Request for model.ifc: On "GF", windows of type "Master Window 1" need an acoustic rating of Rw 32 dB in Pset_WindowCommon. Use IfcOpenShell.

First a look at what the model holds.

```python
import ifcopenshell
import ifcopenshell.util.element

model = ifcopenshell.open("model.ifc")
print(model.schema)
storey = next(s for s in model.by_type("IfcBuildingStorey") if s.Name == "GF")
windows = [e for e in ifcopenshell.util.element.get_decomposition(storey) if e.is_a("IfcWindow")]
seen = {}
for e in windows:
    element_type = ifcopenshell.util.element.get_type(e)
    key = (element_type.Name if element_type != e and element_type else None, ifcopenshell.util.element.get_pset(e, "Pset_WindowCommon", "AcousticRating"))
    seen[key] = seen.get(key, 0) + 1
for (name, value), count in sorted(seen.items(), key=str):
    print(count, "x", name, "|", value)
```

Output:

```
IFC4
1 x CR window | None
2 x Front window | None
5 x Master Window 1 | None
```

```python
import ifcopenshell
import ifcopenshell.api.pset
import ifcopenshell.util.element

model = ifcopenshell.open("model.ifc")

storey = next(s for s in model.by_type("IfcBuildingStorey") if s.Name == "GF")
windows = [e for e in ifcopenshell.util.element.get_decomposition(storey) if e.is_a("IfcWindow")]

count = 0
for e in windows:
    element_type = ifcopenshell.util.element.get_type(e)
    if element_type in (None, e) or element_type.Name != "Master Window 1":
        continue
    # add_pset returns the element's existing set when there is one.
    pset = ifcopenshell.api.pset.add_pset(model, product=e, name="Pset_WindowCommon")
    ifcopenshell.api.pset.edit_pset(model, pset=pset, properties={"AcousticRating": "Rw 32 dB"})
    count += 1

print(count, "windows updated")

model.write("model_edited.ifc")
```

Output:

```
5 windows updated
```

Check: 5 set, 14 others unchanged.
